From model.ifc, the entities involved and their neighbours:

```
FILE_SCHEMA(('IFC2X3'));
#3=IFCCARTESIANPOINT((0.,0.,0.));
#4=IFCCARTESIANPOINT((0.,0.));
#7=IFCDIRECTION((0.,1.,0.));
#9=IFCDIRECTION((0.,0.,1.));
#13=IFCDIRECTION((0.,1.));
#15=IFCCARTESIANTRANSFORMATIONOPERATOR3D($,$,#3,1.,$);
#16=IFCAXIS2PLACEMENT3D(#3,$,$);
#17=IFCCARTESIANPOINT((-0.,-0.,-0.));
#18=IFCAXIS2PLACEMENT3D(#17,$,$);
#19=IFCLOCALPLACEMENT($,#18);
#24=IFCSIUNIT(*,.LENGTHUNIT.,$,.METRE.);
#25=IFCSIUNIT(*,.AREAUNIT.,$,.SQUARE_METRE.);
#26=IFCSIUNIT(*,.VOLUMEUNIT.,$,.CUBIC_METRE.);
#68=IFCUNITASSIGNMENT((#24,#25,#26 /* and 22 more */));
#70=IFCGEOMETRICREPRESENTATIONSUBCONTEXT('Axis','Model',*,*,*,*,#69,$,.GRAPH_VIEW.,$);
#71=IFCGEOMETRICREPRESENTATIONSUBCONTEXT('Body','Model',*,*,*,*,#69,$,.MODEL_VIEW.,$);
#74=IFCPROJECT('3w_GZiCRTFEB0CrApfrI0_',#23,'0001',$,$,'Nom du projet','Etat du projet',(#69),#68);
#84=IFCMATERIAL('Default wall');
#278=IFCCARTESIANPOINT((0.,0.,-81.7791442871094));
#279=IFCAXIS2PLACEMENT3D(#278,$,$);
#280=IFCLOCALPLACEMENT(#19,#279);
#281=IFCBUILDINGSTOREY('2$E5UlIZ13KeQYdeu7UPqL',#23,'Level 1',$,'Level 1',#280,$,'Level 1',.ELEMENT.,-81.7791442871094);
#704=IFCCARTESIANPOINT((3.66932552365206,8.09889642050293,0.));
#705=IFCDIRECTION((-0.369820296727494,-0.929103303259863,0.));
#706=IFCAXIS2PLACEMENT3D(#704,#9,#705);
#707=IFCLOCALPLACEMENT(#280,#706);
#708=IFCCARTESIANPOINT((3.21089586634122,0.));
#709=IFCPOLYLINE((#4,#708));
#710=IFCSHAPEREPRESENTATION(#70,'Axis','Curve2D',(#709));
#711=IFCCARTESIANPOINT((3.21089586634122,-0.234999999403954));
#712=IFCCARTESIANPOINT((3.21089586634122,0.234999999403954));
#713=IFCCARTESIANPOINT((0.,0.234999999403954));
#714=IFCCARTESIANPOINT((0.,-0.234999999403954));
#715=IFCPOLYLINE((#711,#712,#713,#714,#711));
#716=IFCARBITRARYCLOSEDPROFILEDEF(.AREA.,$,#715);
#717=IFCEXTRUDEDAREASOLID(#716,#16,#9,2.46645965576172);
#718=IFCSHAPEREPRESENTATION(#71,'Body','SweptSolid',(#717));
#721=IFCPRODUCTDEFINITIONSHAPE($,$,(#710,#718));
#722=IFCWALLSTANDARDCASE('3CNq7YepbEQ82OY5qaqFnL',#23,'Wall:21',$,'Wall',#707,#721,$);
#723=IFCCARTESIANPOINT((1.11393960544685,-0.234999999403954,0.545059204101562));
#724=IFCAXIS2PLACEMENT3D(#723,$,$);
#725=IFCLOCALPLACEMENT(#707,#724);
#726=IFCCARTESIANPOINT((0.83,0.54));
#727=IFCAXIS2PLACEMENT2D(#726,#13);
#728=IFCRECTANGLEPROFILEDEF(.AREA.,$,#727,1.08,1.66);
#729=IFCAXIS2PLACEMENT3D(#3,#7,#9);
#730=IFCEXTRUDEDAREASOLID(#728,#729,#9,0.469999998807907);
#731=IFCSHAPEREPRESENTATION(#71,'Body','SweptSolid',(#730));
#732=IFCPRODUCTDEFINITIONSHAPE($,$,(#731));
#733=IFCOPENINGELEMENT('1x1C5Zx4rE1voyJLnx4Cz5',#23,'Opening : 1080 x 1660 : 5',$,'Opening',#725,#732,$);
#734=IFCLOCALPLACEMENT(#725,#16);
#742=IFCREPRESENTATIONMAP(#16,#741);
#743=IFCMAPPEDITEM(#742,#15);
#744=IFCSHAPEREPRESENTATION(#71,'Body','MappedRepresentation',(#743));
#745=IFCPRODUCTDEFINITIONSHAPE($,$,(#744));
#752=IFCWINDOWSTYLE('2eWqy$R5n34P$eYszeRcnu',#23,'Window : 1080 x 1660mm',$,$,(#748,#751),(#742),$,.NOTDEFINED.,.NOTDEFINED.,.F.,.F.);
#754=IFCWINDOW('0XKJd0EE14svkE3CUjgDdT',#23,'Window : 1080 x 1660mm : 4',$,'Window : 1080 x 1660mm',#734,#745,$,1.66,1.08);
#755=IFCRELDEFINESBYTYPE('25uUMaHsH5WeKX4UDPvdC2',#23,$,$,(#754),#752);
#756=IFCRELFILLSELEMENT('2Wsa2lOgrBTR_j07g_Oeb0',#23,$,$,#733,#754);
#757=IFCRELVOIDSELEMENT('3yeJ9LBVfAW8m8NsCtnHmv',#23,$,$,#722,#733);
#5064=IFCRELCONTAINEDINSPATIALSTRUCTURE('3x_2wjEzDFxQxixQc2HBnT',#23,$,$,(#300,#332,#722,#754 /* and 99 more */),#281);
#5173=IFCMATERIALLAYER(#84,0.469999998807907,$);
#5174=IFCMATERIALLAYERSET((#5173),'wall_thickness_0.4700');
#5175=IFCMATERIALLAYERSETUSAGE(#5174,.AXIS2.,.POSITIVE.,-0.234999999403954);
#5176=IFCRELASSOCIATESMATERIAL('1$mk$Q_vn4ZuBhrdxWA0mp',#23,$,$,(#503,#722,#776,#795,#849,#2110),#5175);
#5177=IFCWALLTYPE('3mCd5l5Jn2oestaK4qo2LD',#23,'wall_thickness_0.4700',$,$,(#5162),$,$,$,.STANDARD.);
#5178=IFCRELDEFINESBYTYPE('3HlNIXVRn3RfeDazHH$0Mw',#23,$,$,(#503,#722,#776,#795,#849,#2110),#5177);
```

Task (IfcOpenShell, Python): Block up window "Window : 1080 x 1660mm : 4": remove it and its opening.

```python
import ifcopenshell
import ifcopenshell.api.feature
import ifcopenshell.api.root
import ifcopenshell.geom
import ifcopenshell.util.shape

model = ifcopenshell.open("model.ifc")
settings = ifcopenshell.geom.settings()


def volume(element):
    """Net volume in cubic metres, openings subtracted."""
    shape = ifcopenshell.geom.create_shape(settings, element)
    return ifcopenshell.util.shape.get_volume(shape.geometry)


window = model.by_id(754)
opening = window.FillsVoids[0].RelatingOpeningElement
wall = opening.VoidsElements[0].RelatingBuildingElement
before = volume(wall)

ifcopenshell.api.root.remove_product(model, product=window)
ifcopenshell.api.feature.remove_feature(model, feature=opening)

after = volume(wall)

print(f"wall volume {before:.3f} -> {after:.3f} m3")

model.write("model_v2.ifc")
```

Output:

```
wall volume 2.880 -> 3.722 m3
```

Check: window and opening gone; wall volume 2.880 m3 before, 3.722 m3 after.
